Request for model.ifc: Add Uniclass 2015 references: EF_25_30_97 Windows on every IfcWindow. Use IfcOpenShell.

First a look at what the model holds.

```python
import ifcopenshell

model = ifcopenshell.open("model.ifc")
print(model.schema)
print("classifications:", [c.Name for c in model.by_type("IfcClassification")])
for ifc_class in ("IfcDoor", "IfcRoof", "IfcStair", "IfcWall", "IfcWindow"):
    print(ifc_class, len(model.by_type(ifc_class)))
```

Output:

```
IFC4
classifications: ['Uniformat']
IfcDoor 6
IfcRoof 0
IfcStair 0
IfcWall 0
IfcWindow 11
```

```python
import ifcopenshell
import ifcopenshell.api.classification

model = ifcopenshell.open("model.ifc")

system = ifcopenshell.api.classification.add_classification(model, classification="Uniclass 2015")

codes = {
    "IfcWindow": ("EF_25_30_97", "Windows"),
}
for ifc_class, (code, name) in codes.items():
    products = model.by_type(ifc_class)
    ifcopenshell.api.classification.add_reference(
        model, products=products, classification=system, identification=code, name=name
    )
    print(code, len(products))

model.write("model-out.ifc")
```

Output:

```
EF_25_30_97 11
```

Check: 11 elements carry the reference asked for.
